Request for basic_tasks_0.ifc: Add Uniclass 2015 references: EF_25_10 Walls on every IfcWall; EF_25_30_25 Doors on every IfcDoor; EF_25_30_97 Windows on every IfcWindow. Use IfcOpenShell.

First a look at what the model holds.

```python
import ifcopenshell

model = ifcopenshell.open("basic_tasks_0.ifc")
print(model.schema)
print("classifications:", [c.Name for c in model.by_type("IfcClassification")])
for ifc_class in ("IfcDoor", "IfcRoof", "IfcStair", "IfcWall", "IfcWindow"):
    print(ifc_class, len(model.by_type(ifc_class)))
```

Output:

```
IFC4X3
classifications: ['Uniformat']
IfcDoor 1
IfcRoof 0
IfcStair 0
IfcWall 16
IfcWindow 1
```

```python
import ifcopenshell
import ifcopenshell.api.classification

model = ifcopenshell.open("basic_tasks_0.ifc")

system = ifcopenshell.api.classification.add_classification(model, classification="Uniclass 2015")

codes = {
    "IfcWall": ("EF_25_10", "Walls"),
    "IfcDoor": ("EF_25_30_25", "Doors"),
    "IfcWindow": ("EF_25_30_97", "Windows"),
}
for ifc_class, (code, name) in codes.items():
    products = model.by_type(ifc_class)
    ifcopenshell.api.classification.add_reference(
        model, products=products, classification=system, identification=code, name=name
    )
    print(code, len(products))

model.write("basic_tasks_0-out.ifc")
```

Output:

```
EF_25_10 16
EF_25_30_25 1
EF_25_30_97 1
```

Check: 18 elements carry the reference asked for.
